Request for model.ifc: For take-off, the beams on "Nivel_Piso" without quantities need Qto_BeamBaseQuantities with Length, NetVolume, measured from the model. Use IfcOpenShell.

First a look at what the model holds.

```python
import ifcopenshell
import ifcopenshell.util.element
import ifcopenshell.util.unit

model = ifcopenshell.open("model.ifc")
print(model.schema)
for unit_type in ("LENGTHUNIT", "AREAUNIT", "VOLUMEUNIT"):
    print(unit_type, ifcopenshell.util.unit.calculate_unit_scale(model, unit_type))
storey = next(s for s in model.by_type("IfcBuildingStorey") if s.Name == "Nivel_Piso")
beams = [e for e in ifcopenshell.util.element.get_decomposition(storey) if e.is_a("IfcBeam")]
for e in sorted(beams, key=lambda e: e.id()):
    print(e.id(), e.is_a(), e.Name, list(ifcopenshell.util.element.get_psets(e, qtos_only=True)), sep=" | ")
```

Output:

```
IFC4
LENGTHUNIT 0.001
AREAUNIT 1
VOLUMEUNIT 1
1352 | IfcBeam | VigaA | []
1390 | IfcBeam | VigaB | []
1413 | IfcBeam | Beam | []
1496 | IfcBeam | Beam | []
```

```python
import ifcopenshell
import ifcopenshell.api.pset
import ifcopenshell.geom
import ifcopenshell.util.element
import ifcopenshell.util.shape
import ifcopenshell.util.unit

model = ifcopenshell.open("model.ifc")
unit_scale = ifcopenshell.util.unit.calculate_unit_scale(model)
volume_scale = ifcopenshell.util.unit.calculate_unit_scale(model, "VOLUMEUNIT")
settings = ifcopenshell.geom.settings()

storey = next(s for s in model.by_type("IfcBuildingStorey") if s.Name == "Nivel_Piso")
beams = [e for e in ifcopenshell.util.element.get_decomposition(storey) if e.is_a("IfcBeam")]

for e in sorted(beams, key=lambda e: e.id()):
    if ifcopenshell.util.element.get_psets(e, qtos_only=True, should_inherit=False):
        continue
    # Geometry comes back in metres, in the element's own axes.
    shape = ifcopenshell.geom.create_shape(settings, e)
    values = {
        "Length": ifcopenshell.util.shape.get_max_xyz(shape.geometry) / unit_scale,
        "NetVolume": ifcopenshell.util.shape.get_volume(shape.geometry) / volume_scale,
    }
    qto = ifcopenshell.api.pset.add_qto(model, product=e, name="Qto_BeamBaseQuantities")
    ifcopenshell.api.pset.edit_qto(model, qto=qto, properties=values)
    print(e.id(), {k: round(v, 3) for k, v in values.items()})

model.write("model-out.ifc")
```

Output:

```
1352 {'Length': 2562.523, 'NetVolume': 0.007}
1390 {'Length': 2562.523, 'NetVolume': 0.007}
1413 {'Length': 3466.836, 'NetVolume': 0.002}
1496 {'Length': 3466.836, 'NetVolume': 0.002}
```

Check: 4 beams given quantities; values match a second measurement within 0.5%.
